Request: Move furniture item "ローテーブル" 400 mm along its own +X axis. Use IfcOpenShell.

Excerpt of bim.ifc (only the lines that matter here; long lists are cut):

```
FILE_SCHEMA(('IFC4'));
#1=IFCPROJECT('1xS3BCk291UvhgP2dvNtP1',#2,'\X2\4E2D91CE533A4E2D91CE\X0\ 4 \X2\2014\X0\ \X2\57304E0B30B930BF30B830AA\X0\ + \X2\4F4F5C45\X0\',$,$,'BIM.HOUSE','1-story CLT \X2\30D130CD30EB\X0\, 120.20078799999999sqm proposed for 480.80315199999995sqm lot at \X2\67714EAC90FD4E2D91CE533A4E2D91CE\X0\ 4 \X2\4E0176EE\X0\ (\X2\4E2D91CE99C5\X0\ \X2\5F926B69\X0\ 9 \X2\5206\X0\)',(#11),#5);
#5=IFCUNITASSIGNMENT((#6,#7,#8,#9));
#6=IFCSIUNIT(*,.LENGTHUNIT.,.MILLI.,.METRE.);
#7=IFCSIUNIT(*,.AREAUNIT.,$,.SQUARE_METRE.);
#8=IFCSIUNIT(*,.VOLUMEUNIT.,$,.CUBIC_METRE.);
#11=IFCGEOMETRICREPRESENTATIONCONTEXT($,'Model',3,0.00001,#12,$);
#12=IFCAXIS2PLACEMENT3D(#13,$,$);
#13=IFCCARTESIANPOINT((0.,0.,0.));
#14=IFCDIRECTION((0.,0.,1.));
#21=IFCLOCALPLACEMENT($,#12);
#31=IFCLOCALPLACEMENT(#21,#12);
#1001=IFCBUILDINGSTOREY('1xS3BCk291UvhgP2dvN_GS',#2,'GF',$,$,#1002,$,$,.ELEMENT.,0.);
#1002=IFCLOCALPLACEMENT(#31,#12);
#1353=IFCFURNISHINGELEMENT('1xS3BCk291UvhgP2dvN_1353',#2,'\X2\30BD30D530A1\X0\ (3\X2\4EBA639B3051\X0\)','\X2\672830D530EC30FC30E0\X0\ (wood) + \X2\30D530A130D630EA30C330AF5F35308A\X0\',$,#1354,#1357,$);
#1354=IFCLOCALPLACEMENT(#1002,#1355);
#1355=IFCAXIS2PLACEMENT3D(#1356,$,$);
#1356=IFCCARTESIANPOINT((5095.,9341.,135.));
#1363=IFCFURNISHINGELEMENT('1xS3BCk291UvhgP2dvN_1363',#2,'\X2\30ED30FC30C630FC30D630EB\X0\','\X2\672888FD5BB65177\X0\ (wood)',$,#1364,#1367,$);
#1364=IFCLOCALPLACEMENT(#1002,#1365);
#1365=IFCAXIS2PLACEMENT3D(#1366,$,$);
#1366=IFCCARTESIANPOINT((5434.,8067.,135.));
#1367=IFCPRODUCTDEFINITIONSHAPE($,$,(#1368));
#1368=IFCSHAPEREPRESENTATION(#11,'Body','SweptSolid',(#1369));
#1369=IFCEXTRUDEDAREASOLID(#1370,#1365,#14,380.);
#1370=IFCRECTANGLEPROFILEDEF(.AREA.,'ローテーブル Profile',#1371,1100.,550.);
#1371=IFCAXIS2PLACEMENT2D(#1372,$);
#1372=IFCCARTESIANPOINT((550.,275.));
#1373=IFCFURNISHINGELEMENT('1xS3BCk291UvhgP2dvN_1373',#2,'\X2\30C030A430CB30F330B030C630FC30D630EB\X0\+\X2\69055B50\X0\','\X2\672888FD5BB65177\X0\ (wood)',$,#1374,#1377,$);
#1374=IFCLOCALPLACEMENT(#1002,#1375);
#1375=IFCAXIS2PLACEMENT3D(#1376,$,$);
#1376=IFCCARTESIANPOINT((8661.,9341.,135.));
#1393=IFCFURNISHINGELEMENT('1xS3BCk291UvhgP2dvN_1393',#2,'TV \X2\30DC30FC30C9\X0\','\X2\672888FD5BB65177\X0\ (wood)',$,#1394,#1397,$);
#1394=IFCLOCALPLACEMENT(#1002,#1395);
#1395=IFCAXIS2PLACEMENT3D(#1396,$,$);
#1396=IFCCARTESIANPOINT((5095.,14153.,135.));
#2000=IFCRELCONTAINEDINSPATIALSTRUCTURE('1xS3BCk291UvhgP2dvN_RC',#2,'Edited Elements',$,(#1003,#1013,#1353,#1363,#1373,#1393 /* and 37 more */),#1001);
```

```python
import ifcopenshell
import ifcopenshell.api.geometry
import ifcopenshell.util.placement
import ifcopenshell.util.unit

model = ifcopenshell.open("bim.ifc")
unit_scale = ifcopenshell.util.unit.calculate_unit_scale(model)

item = model.by_guid("1xS3BCk291UvhgP2dvN_1363")
matrix = ifcopenshell.util.placement.get_local_placement(item.ObjectPlacement)
matrix[:3, 3] += matrix[:3, 0] * 0.4 / unit_scale
ifcopenshell.api.geometry.edit_object_placement(model, product=item, matrix=matrix, is_si=False)

print(ifcopenshell.util.placement.get_local_placement(item.ObjectPlacement).round(3) + 0.0)

model.write("bim_v2.ifc")
```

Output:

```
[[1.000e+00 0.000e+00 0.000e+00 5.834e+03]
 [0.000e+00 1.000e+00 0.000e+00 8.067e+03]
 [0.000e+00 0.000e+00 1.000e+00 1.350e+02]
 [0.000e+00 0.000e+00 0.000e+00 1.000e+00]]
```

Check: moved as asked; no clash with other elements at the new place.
